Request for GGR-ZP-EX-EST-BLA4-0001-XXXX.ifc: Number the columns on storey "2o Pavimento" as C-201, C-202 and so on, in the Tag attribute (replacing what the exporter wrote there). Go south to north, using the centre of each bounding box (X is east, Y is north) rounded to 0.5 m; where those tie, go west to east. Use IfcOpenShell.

First a look at what the model holds.

```python
import ifcopenshell
import ifcopenshell.util.element
import ifcopenshell.util.placement

model = ifcopenshell.open("GGR-ZP-EX-EST-BLA4-0001-XXXX.ifc")
print(model.schema)
storey = next(s for s in model.by_type("IfcBuildingStorey") if s.Name == "2o Pavimento")
columns = [e for e in ifcopenshell.util.element.get_decomposition(storey) if e.is_a("IfcColumn")]
for e in sorted(columns, key=lambda e: e.id()):
    origin = ifcopenshell.util.placement.get_local_placement(e.ObjectPlacement)[:3, 3]
    print(e.id(), e.Tag, e.Name, origin.round(2) + 0.0, sep=" | ")
```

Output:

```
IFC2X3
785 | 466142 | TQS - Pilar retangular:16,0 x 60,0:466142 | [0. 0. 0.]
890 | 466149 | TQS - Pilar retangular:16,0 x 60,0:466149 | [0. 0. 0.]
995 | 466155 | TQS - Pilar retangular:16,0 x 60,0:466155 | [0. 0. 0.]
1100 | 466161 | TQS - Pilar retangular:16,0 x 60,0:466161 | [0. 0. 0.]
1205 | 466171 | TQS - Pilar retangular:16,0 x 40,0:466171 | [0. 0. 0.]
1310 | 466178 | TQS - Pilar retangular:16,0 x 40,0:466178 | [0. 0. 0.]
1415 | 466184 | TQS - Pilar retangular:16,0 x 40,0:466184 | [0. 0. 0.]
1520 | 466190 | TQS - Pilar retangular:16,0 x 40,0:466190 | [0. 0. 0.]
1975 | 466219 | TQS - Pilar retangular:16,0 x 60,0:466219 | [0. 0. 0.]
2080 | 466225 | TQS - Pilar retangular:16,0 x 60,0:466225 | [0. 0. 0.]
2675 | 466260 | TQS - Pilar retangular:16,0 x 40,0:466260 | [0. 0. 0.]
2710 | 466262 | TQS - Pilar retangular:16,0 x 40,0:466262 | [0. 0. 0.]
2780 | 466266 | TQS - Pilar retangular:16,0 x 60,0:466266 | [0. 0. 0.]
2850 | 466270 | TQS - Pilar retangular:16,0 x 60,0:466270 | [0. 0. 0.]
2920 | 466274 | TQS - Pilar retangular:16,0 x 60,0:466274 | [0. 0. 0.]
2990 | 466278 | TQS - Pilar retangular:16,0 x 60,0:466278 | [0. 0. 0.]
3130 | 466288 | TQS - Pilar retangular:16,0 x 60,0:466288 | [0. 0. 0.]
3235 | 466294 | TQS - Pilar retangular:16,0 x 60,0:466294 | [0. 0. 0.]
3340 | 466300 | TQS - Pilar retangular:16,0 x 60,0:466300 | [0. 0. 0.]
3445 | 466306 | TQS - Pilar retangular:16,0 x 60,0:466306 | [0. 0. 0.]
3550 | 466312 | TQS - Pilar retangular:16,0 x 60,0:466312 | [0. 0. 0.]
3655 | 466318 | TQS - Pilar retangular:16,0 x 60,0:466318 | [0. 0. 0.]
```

```python
import ifcopenshell
import ifcopenshell.geom
import ifcopenshell.util.element
import ifcopenshell.util.shape

model = ifcopenshell.open("GGR-ZP-EX-EST-BLA4-0001-XXXX.ifc")
settings = ifcopenshell.geom.settings()
settings.set("use-world-coords", True)


def centre(element):
    shape = ifcopenshell.geom.create_shape(settings, element)
    return ifcopenshell.util.shape.get_bbox_centroid(shape.geometry)


storey = next(s for s in model.by_type("IfcBuildingStorey") if s.Name == "2o Pavimento")
columns = [e for e in ifcopenshell.util.element.get_decomposition(storey) if e.is_a("IfcColumn")]

# Insertion points can sit at a corner or the storey origin, so sort by the geometry (in metres).
centres = {e: centre(e) for e in columns}
columns.sort(key=lambda e: (round(centres[e][1] / 0.5), centres[e][0]))

for i, e in enumerate(columns, start=1):
    number = f"C-2{i:02d}"
    e.Tag = number
    print(e.id(), number)

model.write("GGR-ZP-EX-EST-BLA4-0001-XXXX_updated.ifc")
```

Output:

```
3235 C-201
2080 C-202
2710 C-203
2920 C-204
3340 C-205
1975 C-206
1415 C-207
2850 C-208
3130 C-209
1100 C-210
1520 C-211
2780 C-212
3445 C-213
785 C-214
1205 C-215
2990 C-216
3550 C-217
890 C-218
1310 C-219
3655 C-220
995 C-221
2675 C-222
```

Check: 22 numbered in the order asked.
